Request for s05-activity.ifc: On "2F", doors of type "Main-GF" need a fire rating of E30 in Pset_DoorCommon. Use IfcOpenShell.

First a look at what the model holds.

```python
import ifcopenshell
import ifcopenshell.util.element

model = ifcopenshell.open("s05-activity.ifc")
print(model.schema)
storey = next(s for s in model.by_type("IfcBuildingStorey") if s.Name == "2F")
doors = [e for e in ifcopenshell.util.element.get_decomposition(storey) if e.is_a("IfcDoor")]
seen = {}
for e in doors:
    element_type = ifcopenshell.util.element.get_type(e)
    key = (element_type.Name if element_type != e and element_type else None, ifcopenshell.util.element.get_pset(e, "Pset_DoorCommon", "FireRating"))
    seen[key] = seen.get(key, 0) + 1
for (name, value), count in sorted(seen.items(), key=str):
    print(count, "x", name, "|", value)
```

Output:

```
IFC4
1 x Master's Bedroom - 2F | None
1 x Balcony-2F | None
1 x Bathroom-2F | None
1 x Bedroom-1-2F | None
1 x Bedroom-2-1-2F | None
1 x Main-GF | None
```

```python
import ifcopenshell
import ifcopenshell.api.pset
import ifcopenshell.util.element

model = ifcopenshell.open("s05-activity.ifc")

storey = next(s for s in model.by_type("IfcBuildingStorey") if s.Name == "2F")
doors = [e for e in ifcopenshell.util.element.get_decomposition(storey) if e.is_a("IfcDoor")]

count = 0
for e in doors:
    element_type = ifcopenshell.util.element.get_type(e)
    if element_type in (None, e) or element_type.Name != "Main-GF":
        continue
    # add_pset returns the element's existing set when there is one.
    pset = ifcopenshell.api.pset.add_pset(model, product=e, name="Pset_DoorCommon")
    ifcopenshell.api.pset.edit_pset(model, pset=pset, properties={"FireRating": "E30"})
    count += 1

print(count, "doors updated")

model.write("s05-activity_updated.ifc")
```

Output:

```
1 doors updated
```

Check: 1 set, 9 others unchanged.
